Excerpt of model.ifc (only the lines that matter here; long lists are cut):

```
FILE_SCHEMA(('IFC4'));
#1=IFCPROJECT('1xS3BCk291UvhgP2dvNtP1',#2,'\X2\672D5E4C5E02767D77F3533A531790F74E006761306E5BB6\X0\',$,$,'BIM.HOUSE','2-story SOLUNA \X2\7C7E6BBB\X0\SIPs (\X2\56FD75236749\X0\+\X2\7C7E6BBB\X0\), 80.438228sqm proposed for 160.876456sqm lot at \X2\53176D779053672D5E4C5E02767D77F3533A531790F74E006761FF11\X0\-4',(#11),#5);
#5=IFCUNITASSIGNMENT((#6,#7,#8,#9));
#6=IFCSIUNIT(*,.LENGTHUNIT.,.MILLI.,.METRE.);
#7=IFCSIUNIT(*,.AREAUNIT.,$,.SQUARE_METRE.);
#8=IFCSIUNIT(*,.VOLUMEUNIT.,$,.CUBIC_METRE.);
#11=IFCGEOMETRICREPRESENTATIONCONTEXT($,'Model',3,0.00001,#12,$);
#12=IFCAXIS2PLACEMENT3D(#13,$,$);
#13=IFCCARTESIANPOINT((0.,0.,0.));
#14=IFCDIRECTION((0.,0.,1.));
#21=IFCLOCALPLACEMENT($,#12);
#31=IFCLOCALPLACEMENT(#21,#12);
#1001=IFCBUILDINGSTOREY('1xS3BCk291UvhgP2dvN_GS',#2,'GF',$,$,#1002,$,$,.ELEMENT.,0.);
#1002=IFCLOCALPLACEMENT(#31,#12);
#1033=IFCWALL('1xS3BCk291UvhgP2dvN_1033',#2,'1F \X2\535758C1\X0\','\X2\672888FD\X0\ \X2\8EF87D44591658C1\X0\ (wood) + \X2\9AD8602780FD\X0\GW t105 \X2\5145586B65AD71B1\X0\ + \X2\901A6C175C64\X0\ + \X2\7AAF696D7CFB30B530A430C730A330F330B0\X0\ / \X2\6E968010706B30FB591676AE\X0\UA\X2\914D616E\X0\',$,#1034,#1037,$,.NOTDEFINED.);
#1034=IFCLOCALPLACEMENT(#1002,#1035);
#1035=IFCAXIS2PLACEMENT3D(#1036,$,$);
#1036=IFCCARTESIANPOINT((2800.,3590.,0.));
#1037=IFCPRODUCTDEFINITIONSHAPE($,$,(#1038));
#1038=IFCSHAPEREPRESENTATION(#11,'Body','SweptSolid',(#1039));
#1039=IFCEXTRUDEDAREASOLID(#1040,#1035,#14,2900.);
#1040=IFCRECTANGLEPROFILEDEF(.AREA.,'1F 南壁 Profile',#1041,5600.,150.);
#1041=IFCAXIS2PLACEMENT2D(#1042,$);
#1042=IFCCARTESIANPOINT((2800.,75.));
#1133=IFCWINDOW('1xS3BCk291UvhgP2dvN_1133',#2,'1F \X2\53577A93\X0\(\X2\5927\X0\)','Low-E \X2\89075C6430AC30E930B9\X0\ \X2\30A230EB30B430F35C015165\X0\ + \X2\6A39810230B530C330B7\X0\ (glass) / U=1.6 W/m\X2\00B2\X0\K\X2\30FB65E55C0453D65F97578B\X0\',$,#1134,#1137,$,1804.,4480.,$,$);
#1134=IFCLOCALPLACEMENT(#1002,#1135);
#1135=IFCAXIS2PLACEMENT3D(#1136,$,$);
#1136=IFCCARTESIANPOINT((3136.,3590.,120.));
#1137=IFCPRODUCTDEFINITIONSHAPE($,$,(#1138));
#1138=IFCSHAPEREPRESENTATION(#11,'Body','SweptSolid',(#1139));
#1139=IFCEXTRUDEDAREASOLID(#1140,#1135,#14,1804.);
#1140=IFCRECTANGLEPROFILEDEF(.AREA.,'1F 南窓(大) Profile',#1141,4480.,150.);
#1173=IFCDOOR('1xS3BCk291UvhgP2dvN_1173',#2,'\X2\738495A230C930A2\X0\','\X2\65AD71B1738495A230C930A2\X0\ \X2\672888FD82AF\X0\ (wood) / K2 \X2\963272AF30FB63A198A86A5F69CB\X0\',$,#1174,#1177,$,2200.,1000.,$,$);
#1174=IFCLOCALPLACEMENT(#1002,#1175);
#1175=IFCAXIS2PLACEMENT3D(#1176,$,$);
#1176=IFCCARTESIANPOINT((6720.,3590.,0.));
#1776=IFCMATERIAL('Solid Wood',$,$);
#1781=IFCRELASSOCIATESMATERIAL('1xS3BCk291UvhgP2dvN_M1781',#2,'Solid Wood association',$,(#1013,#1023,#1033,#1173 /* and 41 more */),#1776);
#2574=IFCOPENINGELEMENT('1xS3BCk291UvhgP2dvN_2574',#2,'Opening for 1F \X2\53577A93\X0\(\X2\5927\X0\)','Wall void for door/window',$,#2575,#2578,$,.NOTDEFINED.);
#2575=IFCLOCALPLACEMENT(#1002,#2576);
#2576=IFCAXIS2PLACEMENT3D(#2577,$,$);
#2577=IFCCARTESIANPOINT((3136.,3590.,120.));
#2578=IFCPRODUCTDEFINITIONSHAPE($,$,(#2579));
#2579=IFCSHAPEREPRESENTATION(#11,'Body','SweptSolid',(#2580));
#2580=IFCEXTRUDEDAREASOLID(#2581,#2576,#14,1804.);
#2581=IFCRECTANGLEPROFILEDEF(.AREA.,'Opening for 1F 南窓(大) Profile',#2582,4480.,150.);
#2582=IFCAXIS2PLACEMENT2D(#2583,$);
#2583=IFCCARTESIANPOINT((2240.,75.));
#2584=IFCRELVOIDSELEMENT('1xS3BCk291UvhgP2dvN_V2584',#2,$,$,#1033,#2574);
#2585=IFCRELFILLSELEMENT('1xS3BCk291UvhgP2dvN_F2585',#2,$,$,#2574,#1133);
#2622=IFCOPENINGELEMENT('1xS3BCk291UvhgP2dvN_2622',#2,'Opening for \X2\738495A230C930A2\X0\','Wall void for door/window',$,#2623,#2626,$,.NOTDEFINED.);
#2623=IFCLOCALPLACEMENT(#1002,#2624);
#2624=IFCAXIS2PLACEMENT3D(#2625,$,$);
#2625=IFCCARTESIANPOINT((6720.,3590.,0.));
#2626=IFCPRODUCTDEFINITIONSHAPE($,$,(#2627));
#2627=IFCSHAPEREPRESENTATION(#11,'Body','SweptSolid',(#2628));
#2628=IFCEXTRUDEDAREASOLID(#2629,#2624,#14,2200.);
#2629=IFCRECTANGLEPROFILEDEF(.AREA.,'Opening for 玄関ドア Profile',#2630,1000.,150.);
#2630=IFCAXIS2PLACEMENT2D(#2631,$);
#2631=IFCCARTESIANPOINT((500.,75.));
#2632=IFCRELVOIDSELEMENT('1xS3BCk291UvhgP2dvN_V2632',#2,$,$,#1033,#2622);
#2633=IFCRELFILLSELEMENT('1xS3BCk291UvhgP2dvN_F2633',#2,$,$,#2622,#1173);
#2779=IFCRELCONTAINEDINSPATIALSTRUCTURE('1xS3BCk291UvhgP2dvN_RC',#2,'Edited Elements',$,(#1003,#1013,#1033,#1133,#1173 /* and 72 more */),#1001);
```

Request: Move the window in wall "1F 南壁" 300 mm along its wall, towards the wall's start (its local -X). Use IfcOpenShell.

```python
import ifcopenshell
import ifcopenshell.api.geometry
import ifcopenshell.util.placement

model = ifcopenshell.open("model.ifc")

window = model.by_id(1133)
opening = window.FillsVoids[0].RelatingOpeningElement
wall = opening.VoidsElements[0].RelatingBuildingElement

wall_matrix = ifcopenshell.util.placement.get_local_placement(wall.ObjectPlacement)
shift = wall_matrix[:3, 0] * -300.0
before = ifcopenshell.util.placement.get_local_placement(window.ObjectPlacement)[:3, 3].copy()

# The window is not placed relative to its opening, so move both.
for product in (opening, window):
    matrix = ifcopenshell.util.placement.get_local_placement(product.ObjectPlacement)
    matrix[:3, 3] += shift
    ifcopenshell.api.geometry.edit_object_placement(model, product=product, matrix=matrix, is_si=False)

after = ifcopenshell.util.placement.get_local_placement(window.ObjectPlacement)[:3, 3]
print("window moved by", (after - before).round(3) + 0.0)

model.write("model_rev.ifc")
```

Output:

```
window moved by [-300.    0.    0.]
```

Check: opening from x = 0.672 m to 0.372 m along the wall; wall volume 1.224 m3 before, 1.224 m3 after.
